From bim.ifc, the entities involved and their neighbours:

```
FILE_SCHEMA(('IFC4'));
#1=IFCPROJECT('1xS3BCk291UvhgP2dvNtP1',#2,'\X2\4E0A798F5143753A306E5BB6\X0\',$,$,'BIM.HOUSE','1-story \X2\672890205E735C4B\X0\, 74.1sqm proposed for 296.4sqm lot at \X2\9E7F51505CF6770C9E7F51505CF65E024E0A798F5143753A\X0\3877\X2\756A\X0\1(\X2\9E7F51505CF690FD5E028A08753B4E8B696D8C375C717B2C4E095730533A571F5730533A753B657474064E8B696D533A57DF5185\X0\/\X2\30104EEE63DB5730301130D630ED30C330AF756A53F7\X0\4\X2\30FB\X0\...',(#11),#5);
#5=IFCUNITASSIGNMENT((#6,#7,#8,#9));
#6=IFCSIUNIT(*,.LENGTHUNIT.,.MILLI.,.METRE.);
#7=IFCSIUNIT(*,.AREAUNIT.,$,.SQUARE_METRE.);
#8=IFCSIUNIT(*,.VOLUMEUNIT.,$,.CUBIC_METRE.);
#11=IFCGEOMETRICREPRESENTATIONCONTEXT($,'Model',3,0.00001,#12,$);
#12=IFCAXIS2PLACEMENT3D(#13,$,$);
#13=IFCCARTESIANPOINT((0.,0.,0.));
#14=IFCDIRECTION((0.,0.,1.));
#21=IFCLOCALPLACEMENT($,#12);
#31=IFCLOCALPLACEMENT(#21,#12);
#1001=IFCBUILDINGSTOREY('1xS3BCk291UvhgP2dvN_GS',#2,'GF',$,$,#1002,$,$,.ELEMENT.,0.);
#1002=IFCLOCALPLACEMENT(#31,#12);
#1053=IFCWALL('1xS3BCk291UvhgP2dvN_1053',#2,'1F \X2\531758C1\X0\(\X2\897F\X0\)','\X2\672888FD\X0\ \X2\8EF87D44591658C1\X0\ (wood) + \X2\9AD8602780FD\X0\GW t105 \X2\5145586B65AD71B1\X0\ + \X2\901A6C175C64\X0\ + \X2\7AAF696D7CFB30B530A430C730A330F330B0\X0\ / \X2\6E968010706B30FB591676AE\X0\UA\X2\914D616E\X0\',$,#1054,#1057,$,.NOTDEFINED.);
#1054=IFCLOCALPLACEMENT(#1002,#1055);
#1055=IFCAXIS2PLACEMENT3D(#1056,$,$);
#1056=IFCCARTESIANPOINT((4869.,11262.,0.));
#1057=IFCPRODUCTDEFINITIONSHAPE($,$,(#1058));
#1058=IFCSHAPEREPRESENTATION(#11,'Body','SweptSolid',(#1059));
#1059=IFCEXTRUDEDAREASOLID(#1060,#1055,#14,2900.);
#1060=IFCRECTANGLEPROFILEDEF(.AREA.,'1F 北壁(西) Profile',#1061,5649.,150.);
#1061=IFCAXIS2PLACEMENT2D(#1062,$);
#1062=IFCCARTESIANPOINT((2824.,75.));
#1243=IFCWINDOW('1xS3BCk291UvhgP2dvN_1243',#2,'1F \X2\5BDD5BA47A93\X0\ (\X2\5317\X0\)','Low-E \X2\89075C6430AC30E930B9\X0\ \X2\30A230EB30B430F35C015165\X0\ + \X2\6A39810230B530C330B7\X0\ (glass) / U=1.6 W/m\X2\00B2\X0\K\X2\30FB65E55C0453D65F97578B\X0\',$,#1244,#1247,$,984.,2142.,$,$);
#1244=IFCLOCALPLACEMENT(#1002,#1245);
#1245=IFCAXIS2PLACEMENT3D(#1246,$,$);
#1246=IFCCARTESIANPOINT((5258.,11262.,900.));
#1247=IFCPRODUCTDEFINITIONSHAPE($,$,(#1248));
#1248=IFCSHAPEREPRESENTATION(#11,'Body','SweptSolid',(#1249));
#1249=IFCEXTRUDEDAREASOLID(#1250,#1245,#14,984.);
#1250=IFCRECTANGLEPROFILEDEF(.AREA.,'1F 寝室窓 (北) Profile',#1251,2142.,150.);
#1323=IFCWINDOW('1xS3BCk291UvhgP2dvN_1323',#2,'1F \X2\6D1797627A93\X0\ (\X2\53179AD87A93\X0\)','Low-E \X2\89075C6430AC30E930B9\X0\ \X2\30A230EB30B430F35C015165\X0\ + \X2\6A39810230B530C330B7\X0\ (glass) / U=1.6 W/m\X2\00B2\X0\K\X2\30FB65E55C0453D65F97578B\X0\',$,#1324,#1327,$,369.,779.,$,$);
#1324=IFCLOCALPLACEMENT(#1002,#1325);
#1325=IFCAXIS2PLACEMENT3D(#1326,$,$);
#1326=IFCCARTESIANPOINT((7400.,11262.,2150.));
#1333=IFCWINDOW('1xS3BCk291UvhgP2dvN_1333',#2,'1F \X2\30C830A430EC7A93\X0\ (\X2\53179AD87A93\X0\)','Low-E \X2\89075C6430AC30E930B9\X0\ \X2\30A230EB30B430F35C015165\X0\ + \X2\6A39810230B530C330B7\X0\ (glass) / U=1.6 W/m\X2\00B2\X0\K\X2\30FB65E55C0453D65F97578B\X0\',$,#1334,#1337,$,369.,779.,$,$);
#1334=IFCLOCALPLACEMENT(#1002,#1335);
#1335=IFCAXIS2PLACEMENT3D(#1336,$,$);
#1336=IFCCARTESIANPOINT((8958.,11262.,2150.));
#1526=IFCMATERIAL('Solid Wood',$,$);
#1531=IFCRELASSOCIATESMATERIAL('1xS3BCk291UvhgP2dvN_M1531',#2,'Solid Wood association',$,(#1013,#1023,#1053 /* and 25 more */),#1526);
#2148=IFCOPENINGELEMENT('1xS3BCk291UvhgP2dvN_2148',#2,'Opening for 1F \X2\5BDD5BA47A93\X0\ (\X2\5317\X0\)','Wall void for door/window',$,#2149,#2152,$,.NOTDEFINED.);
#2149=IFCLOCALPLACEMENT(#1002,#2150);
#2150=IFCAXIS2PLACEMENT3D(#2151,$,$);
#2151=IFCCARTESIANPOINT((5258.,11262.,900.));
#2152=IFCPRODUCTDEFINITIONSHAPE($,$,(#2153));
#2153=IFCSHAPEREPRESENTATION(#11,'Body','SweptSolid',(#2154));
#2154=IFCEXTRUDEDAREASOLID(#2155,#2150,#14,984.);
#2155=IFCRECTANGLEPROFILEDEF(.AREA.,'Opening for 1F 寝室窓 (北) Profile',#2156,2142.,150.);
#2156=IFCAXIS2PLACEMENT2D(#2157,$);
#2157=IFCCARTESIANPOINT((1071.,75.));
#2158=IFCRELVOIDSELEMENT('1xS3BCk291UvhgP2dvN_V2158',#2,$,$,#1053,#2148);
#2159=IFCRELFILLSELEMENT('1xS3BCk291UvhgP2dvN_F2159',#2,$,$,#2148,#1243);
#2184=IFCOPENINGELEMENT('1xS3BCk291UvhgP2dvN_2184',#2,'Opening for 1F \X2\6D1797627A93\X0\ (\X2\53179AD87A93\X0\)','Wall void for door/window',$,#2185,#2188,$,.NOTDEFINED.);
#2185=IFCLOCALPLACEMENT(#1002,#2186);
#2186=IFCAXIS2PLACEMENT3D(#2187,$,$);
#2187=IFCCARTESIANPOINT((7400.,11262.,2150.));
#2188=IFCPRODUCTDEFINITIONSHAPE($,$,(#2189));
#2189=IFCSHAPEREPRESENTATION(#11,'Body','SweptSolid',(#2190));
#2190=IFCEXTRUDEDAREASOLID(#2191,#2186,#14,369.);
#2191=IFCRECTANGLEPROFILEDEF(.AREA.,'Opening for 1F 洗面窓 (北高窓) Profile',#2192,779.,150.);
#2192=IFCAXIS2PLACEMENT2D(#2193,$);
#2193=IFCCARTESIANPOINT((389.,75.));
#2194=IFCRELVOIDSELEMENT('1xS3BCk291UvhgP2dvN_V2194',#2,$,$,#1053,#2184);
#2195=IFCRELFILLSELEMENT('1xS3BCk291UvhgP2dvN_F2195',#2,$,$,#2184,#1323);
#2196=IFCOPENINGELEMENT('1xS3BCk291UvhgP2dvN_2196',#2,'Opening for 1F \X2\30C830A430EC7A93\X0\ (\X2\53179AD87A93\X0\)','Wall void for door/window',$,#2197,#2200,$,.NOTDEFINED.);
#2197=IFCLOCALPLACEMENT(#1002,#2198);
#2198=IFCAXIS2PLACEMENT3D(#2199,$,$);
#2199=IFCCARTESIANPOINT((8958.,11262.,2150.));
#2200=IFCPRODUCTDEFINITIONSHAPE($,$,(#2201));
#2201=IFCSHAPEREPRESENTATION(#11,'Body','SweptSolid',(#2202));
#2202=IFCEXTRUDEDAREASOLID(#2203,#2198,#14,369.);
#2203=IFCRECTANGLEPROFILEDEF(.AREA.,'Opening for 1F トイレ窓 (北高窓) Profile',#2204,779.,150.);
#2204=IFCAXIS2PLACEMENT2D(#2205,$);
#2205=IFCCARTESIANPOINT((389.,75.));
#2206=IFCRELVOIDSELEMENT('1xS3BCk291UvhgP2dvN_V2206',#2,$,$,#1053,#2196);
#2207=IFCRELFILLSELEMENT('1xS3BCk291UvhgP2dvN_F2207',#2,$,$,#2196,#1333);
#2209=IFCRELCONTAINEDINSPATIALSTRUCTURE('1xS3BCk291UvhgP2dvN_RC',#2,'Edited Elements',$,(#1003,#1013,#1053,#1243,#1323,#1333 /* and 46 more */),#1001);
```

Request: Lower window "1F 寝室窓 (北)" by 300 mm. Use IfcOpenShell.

```python
import numpy as np
import ifcopenshell
import ifcopenshell.api.geometry
import ifcopenshell.util.placement
import ifcopenshell.util.unit

model = ifcopenshell.open("bim.ifc")
unit_scale = ifcopenshell.util.unit.calculate_unit_scale(model)

window = model.by_id(1243)
opening = window.FillsVoids[0].RelatingOpeningElement
dz = -300.0

shift = np.array([0.0, 0.0, dz])
# The window is not placed relative to its opening, so move both.
for product in (opening, window):
    matrix = ifcopenshell.util.placement.get_local_placement(product.ObjectPlacement)
    matrix[:3, 3] += shift
    ifcopenshell.api.geometry.edit_object_placement(model, product=product, matrix=matrix, is_si=False)

print(f"moved by {dz * unit_scale:+.3f} m")

model.write("bim_rev.ifc")
```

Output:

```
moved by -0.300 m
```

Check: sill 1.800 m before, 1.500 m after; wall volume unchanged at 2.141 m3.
